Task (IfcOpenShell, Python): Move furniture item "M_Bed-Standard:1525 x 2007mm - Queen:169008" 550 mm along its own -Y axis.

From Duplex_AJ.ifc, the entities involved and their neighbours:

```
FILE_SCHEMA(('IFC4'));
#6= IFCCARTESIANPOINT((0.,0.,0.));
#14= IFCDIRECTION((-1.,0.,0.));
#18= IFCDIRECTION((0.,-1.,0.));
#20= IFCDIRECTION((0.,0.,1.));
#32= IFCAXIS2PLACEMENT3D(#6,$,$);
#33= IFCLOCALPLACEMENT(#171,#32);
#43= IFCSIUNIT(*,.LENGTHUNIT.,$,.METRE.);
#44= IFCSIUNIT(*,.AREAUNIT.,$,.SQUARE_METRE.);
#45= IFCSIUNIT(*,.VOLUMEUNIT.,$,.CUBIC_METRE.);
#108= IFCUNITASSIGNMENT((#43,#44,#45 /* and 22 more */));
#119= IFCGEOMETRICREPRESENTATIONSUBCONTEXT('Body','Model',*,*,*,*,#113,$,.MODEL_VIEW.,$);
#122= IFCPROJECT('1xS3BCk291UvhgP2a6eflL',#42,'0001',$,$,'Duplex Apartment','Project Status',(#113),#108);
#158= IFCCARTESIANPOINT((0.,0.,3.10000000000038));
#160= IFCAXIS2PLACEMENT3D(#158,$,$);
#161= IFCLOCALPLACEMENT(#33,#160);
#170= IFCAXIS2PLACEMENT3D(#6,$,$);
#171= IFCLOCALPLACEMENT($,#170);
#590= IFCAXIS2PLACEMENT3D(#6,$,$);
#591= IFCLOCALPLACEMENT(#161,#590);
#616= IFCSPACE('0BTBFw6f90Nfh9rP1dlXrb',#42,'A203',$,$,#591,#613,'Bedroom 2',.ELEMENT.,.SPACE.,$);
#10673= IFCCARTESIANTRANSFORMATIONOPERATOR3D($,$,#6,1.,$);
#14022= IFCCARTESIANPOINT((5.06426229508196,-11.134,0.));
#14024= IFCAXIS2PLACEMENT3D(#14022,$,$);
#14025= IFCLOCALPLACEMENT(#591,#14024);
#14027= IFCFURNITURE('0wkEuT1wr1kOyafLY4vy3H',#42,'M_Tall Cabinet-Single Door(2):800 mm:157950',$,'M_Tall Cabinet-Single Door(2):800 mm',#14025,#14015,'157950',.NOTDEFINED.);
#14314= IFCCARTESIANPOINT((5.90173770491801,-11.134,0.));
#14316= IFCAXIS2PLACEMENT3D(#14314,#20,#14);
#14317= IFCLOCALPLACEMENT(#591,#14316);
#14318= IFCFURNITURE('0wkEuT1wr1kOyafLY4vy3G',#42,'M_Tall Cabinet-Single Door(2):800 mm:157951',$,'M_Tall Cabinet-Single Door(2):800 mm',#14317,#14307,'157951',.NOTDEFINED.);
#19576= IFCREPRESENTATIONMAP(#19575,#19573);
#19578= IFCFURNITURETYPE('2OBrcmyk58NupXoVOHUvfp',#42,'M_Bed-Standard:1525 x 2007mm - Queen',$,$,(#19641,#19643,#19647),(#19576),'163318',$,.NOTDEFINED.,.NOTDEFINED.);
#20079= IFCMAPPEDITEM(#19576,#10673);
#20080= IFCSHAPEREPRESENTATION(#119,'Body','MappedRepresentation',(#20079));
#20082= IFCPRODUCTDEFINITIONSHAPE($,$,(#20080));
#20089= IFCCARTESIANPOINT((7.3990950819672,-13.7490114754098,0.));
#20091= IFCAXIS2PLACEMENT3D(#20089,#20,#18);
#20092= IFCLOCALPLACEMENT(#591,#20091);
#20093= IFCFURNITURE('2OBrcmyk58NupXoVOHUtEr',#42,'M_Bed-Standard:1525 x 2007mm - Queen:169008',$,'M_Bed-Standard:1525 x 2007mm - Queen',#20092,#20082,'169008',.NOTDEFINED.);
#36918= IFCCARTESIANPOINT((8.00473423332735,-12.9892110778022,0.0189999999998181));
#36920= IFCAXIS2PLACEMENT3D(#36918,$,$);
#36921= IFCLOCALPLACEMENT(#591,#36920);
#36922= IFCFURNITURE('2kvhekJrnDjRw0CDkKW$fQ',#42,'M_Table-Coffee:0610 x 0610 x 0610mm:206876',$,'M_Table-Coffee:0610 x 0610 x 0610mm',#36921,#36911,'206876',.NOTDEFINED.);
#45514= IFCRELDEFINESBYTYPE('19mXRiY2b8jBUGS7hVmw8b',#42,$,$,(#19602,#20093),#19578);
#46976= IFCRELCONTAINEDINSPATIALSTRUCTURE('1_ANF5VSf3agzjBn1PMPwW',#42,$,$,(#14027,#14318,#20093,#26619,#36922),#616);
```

```python
import ifcopenshell
import ifcopenshell.api.geometry
import ifcopenshell.util.placement

model = ifcopenshell.open("Duplex_AJ.ifc")

item = model.by_id(20093)
matrix = ifcopenshell.util.placement.get_local_placement(item.ObjectPlacement)
matrix[:3, 3] -= matrix[:3, 1] * 0.55
ifcopenshell.api.geometry.edit_object_placement(model, product=item, matrix=matrix, is_si=False)

print(ifcopenshell.util.placement.get_local_placement(item.ObjectPlacement).round(3) + 0.0)

model.write("Duplex_AJ_updated.ifc")
```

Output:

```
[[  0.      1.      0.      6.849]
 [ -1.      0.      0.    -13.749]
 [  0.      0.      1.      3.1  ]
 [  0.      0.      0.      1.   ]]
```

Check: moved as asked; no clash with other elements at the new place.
